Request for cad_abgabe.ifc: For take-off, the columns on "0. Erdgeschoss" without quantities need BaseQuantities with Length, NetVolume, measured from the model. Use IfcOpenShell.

First a look at what the model holds.

```python
import ifcopenshell
import ifcopenshell.util.element
import ifcopenshell.util.unit

model = ifcopenshell.open("cad_abgabe.ifc")
print(model.schema)
for unit_type in ("LENGTHUNIT", "AREAUNIT", "VOLUMEUNIT"):
    print(unit_type, ifcopenshell.util.unit.calculate_unit_scale(model, unit_type))
storey = next(s for s in model.by_type("IfcBuildingStorey") if s.Name == "0. Erdgeschoss")
columns = [e for e in ifcopenshell.util.element.get_decomposition(storey) if e.is_a("IfcColumn")]
for e in sorted(columns, key=lambda e: e.id()):
    print(e.id(), e.is_a(), e.Name, list(ifcopenshell.util.element.get_psets(e, qtos_only=True)), sep=" | ")
```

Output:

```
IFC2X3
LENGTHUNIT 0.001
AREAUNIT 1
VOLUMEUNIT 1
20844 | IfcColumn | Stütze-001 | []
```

```python
import ifcopenshell
import ifcopenshell.api.pset
import ifcopenshell.geom
import ifcopenshell.util.element
import ifcopenshell.util.shape
import ifcopenshell.util.unit

model = ifcopenshell.open("cad_abgabe.ifc")
unit_scale = ifcopenshell.util.unit.calculate_unit_scale(model)
volume_scale = ifcopenshell.util.unit.calculate_unit_scale(model, "VOLUMEUNIT")
settings = ifcopenshell.geom.settings()

storey = next(s for s in model.by_type("IfcBuildingStorey") if s.Name == "0. Erdgeschoss")
columns = [e for e in ifcopenshell.util.element.get_decomposition(storey) if e.is_a("IfcColumn")]

for e in sorted(columns, key=lambda e: e.id()):
    if ifcopenshell.util.element.get_psets(e, qtos_only=True, should_inherit=False):
        continue
    # Geometry comes back in metres, in the element's own axes.
    shape = ifcopenshell.geom.create_shape(settings, e)
    values = {
        "Length": ifcopenshell.util.shape.get_z(shape.geometry) / unit_scale,
        "NetVolume": ifcopenshell.util.shape.get_volume(shape.geometry) / volume_scale,
    }
    qto = ifcopenshell.api.pset.add_qto(model, product=e, name="BaseQuantities")
    ifcopenshell.api.pset.edit_qto(model, qto=qto, properties=values)
    print(e.id(), {k: round(v, 3) for k, v in values.items()})

model.write("cad_abgabe_v2.ifc")
```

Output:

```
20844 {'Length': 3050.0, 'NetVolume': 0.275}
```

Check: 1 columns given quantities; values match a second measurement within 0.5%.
